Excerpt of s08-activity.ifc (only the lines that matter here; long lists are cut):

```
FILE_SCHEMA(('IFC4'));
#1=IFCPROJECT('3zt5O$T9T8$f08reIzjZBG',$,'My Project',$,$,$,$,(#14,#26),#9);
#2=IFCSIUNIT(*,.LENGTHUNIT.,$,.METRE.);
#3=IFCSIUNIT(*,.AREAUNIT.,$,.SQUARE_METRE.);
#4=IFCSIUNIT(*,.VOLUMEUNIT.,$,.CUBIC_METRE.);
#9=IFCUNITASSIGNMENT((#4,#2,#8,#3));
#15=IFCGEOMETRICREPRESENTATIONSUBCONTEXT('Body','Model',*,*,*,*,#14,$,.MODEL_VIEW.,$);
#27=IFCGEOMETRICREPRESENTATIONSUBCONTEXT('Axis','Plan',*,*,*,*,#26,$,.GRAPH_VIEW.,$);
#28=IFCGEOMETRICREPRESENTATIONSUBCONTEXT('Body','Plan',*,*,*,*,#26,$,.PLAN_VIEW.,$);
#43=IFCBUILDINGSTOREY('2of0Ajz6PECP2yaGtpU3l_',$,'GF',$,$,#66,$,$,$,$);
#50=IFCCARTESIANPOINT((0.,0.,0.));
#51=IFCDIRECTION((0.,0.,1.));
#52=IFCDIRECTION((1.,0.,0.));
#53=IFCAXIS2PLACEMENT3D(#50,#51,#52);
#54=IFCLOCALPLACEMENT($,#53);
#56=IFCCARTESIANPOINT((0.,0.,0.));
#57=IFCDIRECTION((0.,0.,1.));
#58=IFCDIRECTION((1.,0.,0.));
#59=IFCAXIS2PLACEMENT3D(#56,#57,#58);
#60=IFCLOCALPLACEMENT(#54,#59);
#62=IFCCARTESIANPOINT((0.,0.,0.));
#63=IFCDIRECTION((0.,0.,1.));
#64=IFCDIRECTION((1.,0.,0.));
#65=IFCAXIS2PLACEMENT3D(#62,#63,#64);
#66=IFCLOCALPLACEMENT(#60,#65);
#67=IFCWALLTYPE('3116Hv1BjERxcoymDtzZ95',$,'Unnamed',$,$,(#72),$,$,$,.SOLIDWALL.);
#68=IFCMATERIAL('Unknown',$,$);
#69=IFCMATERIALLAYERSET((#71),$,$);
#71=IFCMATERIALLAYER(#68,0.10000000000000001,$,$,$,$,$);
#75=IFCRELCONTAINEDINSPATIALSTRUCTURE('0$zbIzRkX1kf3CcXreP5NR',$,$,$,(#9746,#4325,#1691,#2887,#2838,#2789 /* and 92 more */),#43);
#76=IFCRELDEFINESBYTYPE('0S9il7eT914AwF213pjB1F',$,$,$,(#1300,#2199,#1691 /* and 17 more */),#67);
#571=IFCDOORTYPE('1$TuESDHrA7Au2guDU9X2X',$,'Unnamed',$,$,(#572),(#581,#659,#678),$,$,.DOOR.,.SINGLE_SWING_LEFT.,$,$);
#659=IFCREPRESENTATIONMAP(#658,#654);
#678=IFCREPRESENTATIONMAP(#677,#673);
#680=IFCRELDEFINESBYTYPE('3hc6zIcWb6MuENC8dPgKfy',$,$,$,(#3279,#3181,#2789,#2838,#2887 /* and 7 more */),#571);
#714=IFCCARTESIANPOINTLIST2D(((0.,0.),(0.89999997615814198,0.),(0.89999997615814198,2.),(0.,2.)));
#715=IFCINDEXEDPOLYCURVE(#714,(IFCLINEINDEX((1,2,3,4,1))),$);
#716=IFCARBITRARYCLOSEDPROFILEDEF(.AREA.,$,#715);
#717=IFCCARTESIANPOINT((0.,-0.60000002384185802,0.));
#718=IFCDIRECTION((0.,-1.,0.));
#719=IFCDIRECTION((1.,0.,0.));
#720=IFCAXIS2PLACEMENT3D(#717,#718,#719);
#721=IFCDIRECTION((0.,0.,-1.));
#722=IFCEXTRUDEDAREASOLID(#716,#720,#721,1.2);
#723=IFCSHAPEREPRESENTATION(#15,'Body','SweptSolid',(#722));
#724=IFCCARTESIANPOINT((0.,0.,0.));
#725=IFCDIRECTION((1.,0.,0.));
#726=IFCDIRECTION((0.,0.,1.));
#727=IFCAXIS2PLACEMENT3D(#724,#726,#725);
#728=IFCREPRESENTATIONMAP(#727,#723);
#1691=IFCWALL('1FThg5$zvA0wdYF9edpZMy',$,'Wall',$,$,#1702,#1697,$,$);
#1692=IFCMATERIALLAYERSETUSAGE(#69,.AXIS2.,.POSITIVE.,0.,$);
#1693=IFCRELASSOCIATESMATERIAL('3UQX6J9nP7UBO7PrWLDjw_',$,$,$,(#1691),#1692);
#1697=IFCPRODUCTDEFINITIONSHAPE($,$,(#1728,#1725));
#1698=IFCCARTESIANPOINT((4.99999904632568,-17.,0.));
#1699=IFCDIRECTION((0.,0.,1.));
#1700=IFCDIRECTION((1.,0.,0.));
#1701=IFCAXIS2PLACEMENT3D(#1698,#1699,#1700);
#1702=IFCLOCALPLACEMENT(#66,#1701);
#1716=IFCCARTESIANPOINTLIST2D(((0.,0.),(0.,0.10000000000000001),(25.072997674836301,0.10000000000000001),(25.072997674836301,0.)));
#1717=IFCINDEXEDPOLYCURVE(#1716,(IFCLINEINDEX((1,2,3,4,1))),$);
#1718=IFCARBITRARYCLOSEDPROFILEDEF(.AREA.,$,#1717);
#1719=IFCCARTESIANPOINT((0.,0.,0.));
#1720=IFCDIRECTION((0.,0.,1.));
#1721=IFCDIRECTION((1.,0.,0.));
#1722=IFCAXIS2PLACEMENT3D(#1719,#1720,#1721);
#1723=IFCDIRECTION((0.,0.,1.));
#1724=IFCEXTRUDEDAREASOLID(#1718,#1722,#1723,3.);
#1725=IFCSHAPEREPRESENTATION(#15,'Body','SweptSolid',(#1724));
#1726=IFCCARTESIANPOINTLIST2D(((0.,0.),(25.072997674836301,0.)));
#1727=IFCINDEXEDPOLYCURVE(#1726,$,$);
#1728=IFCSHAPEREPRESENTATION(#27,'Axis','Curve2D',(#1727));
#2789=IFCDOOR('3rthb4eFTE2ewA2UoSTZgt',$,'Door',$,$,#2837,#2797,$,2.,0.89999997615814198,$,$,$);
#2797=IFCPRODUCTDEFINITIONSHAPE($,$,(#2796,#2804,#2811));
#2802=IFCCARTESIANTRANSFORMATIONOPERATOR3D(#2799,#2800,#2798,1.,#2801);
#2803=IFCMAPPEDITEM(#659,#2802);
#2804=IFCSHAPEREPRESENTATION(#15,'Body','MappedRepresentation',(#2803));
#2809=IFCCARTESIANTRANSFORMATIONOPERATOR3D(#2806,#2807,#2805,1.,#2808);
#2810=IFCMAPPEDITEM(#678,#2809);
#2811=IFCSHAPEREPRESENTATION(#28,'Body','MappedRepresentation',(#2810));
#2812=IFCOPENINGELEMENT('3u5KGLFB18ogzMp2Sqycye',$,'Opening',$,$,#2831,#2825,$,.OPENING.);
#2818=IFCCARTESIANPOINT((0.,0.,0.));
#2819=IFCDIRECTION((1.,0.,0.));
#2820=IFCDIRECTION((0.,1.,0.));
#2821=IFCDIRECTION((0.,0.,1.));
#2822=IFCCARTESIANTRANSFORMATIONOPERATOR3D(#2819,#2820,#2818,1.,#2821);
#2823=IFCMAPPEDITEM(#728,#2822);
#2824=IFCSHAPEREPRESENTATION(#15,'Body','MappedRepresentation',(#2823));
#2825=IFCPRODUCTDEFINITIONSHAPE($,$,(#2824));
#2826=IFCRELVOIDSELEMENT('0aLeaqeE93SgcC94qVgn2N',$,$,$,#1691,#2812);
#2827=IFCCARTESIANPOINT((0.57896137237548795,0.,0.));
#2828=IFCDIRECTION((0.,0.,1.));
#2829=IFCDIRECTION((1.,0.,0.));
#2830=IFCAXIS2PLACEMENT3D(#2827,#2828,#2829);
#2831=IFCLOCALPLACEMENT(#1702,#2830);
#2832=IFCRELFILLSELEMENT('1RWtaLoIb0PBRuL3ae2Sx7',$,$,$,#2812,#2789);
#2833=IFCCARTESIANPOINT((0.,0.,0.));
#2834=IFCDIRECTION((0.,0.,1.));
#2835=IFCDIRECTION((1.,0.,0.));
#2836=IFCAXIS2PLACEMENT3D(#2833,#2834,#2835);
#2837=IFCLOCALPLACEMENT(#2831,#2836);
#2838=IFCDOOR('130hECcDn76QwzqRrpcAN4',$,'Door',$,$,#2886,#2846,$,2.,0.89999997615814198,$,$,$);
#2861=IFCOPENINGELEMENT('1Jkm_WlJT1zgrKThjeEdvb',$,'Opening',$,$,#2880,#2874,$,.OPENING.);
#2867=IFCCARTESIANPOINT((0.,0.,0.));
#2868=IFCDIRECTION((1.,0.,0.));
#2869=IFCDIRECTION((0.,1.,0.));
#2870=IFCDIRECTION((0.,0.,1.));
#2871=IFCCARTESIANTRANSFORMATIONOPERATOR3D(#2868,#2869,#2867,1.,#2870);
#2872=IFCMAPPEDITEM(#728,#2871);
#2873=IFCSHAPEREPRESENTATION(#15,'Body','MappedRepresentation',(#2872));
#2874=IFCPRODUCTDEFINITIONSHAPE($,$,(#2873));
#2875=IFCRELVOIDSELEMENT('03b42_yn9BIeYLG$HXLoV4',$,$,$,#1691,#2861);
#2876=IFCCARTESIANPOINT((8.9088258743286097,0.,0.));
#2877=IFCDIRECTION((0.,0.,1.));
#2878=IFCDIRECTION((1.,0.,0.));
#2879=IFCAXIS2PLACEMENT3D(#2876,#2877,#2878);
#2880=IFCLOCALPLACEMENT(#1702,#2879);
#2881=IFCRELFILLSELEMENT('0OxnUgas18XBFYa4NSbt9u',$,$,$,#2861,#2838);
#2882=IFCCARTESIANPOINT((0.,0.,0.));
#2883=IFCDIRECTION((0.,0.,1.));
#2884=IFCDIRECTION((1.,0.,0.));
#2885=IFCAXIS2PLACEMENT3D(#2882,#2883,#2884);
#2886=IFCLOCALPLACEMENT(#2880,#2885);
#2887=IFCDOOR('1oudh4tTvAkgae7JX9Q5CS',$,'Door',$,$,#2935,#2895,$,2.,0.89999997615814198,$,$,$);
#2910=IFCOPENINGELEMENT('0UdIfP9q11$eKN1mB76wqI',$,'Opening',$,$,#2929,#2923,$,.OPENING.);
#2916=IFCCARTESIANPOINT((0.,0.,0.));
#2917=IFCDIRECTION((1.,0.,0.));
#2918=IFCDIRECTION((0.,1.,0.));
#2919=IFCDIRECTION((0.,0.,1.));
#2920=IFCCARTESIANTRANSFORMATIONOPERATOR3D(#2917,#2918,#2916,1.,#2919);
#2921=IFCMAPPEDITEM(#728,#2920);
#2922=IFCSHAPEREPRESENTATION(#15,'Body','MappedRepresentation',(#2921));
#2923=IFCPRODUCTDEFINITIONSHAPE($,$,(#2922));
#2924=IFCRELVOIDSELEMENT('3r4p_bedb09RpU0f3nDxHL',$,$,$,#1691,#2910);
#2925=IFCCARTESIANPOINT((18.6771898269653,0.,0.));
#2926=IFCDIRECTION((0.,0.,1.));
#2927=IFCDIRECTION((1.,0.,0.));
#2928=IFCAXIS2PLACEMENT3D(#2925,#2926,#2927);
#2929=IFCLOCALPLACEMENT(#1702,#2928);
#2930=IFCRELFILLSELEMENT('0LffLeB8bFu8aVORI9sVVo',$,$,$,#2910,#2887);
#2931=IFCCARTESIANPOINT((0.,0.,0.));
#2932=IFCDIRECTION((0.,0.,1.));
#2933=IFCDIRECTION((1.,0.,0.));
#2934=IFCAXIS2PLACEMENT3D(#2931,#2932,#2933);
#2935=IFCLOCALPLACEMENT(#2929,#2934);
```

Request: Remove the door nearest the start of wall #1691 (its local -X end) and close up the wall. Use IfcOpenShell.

```python
import ifcopenshell
import ifcopenshell.api.feature
import ifcopenshell.api.root
import ifcopenshell.geom
import ifcopenshell.util.shape

model = ifcopenshell.open("s08-activity.ifc")
settings = ifcopenshell.geom.settings()


def volume(element):
    """Net volume in cubic metres, openings subtracted."""
    shape = ifcopenshell.geom.create_shape(settings, element)
    return ifcopenshell.util.shape.get_volume(shape.geometry)


door = model.by_guid("3rthb4eFTE2ewA2UoSTZgt")
opening = door.FillsVoids[0].RelatingOpeningElement
wall = opening.VoidsElements[0].RelatingBuildingElement
before = volume(wall)

ifcopenshell.api.root.remove_product(model, product=door)
ifcopenshell.api.feature.remove_feature(model, feature=opening)

after = volume(wall)

print(f"wall volume {before:.3f} -> {after:.3f} m3")

model.write("s08-activity_v2.ifc")
```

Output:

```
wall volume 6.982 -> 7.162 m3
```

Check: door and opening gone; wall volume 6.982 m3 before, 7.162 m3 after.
